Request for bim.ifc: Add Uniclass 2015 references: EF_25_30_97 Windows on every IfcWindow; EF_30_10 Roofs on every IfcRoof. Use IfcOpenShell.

First a look at what the model holds.

```python
import ifcopenshell

model = ifcopenshell.open("bim.ifc")
print(model.schema)
print("classifications:", [c.Name for c in model.by_type("IfcClassification")])
for ifc_class in ("IfcDoor", "IfcRoof", "IfcStair", "IfcWall", "IfcWindow"):
    print(ifc_class, len(model.by_type(ifc_class)))
```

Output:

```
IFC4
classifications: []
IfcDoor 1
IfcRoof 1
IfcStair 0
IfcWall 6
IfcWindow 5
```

```python
import ifcopenshell
import ifcopenshell.api.classification

model = ifcopenshell.open("bim.ifc")

system = ifcopenshell.api.classification.add_classification(model, classification="Uniclass 2015")

codes = {
    "IfcWindow": ("EF_25_30_97", "Windows"),
    "IfcRoof": ("EF_30_10", "Roofs"),
}
for ifc_class, (code, name) in codes.items():
    products = model.by_type(ifc_class)
    ifcopenshell.api.classification.add_reference(
        model, products=products, classification=system, identification=code, name=name
    )
    print(code, len(products))

model.write("bim_rev.ifc")
```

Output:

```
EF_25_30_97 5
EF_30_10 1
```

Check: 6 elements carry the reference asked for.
